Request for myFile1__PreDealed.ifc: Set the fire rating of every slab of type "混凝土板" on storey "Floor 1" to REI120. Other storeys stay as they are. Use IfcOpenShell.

First a look at what the model holds.

```python
import ifcopenshell
import ifcopenshell.util.element

model = ifcopenshell.open("myFile1__PreDealed.ifc")
print(model.schema)
storey = next(s for s in model.by_type("IfcBuildingStorey") if s.Name == "Floor 1")
slabs = [e for e in ifcopenshell.util.element.get_decomposition(storey) if e.is_a("IfcSlab")]
seen = {}
for e in slabs:
    element_type = ifcopenshell.util.element.get_type(e)
    key = (element_type.Name if element_type != e and element_type else None, ifcopenshell.util.element.get_pset(e, "Pset_SlabCommon", "FireRating"))
    seen[key] = seen.get(key, 0) + 1
for (name, value), count in sorted(seen.items(), key=str):
    print(count, "x", name, "|", value)
```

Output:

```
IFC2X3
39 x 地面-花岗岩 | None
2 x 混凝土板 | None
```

```python
import ifcopenshell
import ifcopenshell.api.pset
import ifcopenshell.util.element

model = ifcopenshell.open("myFile1__PreDealed.ifc")

storey = next(s for s in model.by_type("IfcBuildingStorey") if s.Name == "Floor 1")
slabs = [e for e in ifcopenshell.util.element.get_decomposition(storey) if e.is_a("IfcSlab")]

count = 0
for e in slabs:
    element_type = ifcopenshell.util.element.get_type(e)
    if element_type in (None, e) or element_type.Name != "混凝土板":
        continue
    # add_pset returns the element's existing set when there is one.
    pset = ifcopenshell.api.pset.add_pset(model, product=e, name="Pset_SlabCommon")
    ifcopenshell.api.pset.edit_pset(model, pset=pset, properties={"FireRating": "REI120"})
    count += 1

print(count, "slabs updated")

model.write("myFile1__PreDealed_v2.ifc")
```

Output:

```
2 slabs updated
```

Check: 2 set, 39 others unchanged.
